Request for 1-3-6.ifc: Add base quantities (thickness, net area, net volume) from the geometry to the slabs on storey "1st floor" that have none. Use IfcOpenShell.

First a look at what the model holds.

```python
import ifcopenshell
import ifcopenshell.util.element
import ifcopenshell.util.unit

model = ifcopenshell.open("1-3-6.ifc")
print(model.schema)
for unit_type in ("LENGTHUNIT", "AREAUNIT", "VOLUMEUNIT"):
    print(unit_type, ifcopenshell.util.unit.calculate_unit_scale(model, unit_type))
storey = next(s for s in model.by_type("IfcBuildingStorey") if s.Name == "1st floor")
slabs = [e for e in ifcopenshell.util.element.get_decomposition(storey) if e.is_a("IfcSlab")]
for e in sorted(slabs, key=lambda e: e.id()):
    print(e.id(), e.is_a(), e.Name, list(ifcopenshell.util.element.get_psets(e, qtos_only=True)), sep=" | ")
```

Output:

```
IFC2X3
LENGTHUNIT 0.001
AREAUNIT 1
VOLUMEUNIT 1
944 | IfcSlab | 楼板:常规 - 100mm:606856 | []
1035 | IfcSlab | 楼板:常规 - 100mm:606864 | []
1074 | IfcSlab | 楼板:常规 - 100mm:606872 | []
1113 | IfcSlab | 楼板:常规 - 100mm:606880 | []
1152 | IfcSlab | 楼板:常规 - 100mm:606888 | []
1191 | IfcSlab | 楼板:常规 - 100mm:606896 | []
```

```python
import ifcopenshell
import ifcopenshell.api.pset
import ifcopenshell.geom
import ifcopenshell.util.element
import ifcopenshell.util.shape
import ifcopenshell.util.unit

model = ifcopenshell.open("1-3-6.ifc")
unit_scale = ifcopenshell.util.unit.calculate_unit_scale(model)
area_scale = ifcopenshell.util.unit.calculate_unit_scale(model, "AREAUNIT")
volume_scale = ifcopenshell.util.unit.calculate_unit_scale(model, "VOLUMEUNIT")
settings = ifcopenshell.geom.settings()

storey = next(s for s in model.by_type("IfcBuildingStorey") if s.Name == "1st floor")
slabs = [e for e in ifcopenshell.util.element.get_decomposition(storey) if e.is_a("IfcSlab")]

for e in sorted(slabs, key=lambda e: e.id()):
    if ifcopenshell.util.element.get_psets(e, qtos_only=True, should_inherit=False):
        continue
    # Geometry comes back in metres, in the element's own axes.
    shape = ifcopenshell.geom.create_shape(settings, e)
    values = {
        "Width": ifcopenshell.util.shape.get_z(shape.geometry) / unit_scale,
        "NetArea": ifcopenshell.util.shape.get_footprint_area(shape.geometry) / area_scale,
        "NetVolume": ifcopenshell.util.shape.get_volume(shape.geometry) / volume_scale,
    }
    qto = ifcopenshell.api.pset.add_qto(model, product=e, name="BaseQuantities")
    ifcopenshell.api.pset.edit_qto(model, qto=qto, properties=values)
    print(e.id(), {k: round(v, 3) for k, v in values.items()})

model.write("1-3-6-out.ifc")
```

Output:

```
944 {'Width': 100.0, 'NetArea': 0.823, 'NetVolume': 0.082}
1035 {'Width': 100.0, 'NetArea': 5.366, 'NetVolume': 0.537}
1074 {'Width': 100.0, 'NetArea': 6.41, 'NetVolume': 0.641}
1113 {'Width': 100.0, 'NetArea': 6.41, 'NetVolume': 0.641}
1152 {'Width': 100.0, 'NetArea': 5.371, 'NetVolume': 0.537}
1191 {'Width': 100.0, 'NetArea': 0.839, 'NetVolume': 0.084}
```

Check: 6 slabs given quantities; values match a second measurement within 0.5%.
